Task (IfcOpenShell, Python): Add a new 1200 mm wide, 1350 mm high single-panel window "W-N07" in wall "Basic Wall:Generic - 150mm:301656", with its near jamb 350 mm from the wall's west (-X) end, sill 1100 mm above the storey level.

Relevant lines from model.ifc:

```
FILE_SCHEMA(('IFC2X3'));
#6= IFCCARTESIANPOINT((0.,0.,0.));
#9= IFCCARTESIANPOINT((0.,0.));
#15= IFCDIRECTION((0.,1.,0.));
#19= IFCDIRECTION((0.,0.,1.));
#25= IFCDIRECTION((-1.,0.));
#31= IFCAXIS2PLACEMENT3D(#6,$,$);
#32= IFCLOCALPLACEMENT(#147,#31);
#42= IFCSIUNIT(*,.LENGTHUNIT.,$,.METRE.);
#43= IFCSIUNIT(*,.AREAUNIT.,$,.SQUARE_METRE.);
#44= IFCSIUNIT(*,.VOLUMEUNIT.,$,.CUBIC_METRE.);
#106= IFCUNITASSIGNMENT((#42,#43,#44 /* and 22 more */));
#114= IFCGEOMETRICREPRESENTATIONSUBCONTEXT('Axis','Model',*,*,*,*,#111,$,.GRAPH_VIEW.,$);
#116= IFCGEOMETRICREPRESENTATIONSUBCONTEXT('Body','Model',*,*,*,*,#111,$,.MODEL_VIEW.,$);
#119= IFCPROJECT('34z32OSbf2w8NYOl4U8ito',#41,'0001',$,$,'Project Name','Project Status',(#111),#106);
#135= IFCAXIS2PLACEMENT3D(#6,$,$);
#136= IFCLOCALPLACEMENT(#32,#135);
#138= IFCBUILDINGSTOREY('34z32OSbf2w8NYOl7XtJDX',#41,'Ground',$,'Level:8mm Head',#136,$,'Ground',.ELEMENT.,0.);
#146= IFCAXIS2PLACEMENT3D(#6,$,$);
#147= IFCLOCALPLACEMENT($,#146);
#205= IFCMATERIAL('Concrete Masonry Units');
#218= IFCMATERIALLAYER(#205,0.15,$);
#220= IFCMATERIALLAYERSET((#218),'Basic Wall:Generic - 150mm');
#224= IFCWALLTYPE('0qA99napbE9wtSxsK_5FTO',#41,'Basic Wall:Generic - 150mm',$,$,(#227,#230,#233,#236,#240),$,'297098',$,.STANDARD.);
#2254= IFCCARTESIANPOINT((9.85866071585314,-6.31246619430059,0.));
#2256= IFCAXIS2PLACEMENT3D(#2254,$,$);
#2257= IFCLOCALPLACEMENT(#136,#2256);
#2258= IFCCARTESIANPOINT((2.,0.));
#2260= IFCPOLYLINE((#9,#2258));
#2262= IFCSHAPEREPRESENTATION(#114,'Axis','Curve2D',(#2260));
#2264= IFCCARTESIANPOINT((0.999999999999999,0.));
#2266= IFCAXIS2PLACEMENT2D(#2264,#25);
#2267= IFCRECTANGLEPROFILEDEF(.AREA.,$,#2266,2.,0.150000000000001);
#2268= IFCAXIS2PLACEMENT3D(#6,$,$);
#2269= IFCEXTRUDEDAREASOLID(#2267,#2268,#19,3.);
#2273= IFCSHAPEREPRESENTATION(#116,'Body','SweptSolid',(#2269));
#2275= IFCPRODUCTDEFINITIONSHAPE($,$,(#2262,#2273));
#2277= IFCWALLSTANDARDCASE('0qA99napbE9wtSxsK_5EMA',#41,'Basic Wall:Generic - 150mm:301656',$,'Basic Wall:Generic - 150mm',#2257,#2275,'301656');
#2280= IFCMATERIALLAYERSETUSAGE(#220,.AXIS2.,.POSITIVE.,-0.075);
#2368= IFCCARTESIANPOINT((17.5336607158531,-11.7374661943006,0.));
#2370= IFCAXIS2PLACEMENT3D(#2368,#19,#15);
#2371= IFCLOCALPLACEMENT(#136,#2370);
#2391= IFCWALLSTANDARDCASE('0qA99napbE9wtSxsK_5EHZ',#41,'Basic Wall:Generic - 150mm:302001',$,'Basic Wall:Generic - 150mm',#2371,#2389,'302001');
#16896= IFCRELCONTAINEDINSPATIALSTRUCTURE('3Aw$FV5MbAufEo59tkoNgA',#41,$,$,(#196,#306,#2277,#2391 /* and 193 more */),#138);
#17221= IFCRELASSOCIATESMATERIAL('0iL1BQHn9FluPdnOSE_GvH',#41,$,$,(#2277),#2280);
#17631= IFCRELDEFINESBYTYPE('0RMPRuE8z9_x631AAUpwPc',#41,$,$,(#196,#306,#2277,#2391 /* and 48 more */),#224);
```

```python
import numpy as np
import ifcopenshell
import ifcopenshell.api.feature
import ifcopenshell.api.geometry
import ifcopenshell.api.root
import ifcopenshell.api.spatial
import ifcopenshell.api.type
import ifcopenshell.geom
import ifcopenshell.util.element
import ifcopenshell.util.placement
import ifcopenshell.util.representation
import ifcopenshell.util.shape
import ifcopenshell.util.unit

model = ifcopenshell.open("model.ifc")
unit_scale = ifcopenshell.util.unit.calculate_unit_scale(model)
settings = ifcopenshell.geom.settings()


def volume(element):
    """Net volume in cubic metres, openings subtracted."""
    shape = ifcopenshell.geom.create_shape(settings, element)
    return ifcopenshell.util.shape.get_volume(shape.geometry)


wall = model.by_guid("0qA99napbE9wtSxsK_5EMA")
storey = ifcopenshell.util.element.get_container(wall, ifc_class="IfcBuildingStorey")
context = ifcopenshell.util.representation.get_context(model, "Model", "Body", "MODEL_VIEW")
before = volume(wall)

width, height, from_end, sill = 1.2, 1.35, 0.35, 1.1  # metres

# The wall runs along its own X axis, and the end named is its -X end.
wall_shape = ifcopenshell.geom.create_shape(settings, wall)
x, y, z = ifcopenshell.util.shape.get_vertices(wall_shape.geometry).T
start = x.min() + from_end
face, thickness = float(y.min()), float(y.max() - y.min())
wall_matrix = ifcopenshell.util.placement.get_local_placement(wall.ObjectPlacement)
level = ifcopenshell.util.placement.get_local_placement(storey.ObjectPlacement)[2, 3]


def in_wall(x, y):
    """Placement at x, y metres in the wall's axes, at sill height."""
    matrix = wall_matrix.copy()
    matrix[:, 3] = wall_matrix @ np.array([x / unit_scale, y / unit_scale, 0.0, 1.0])
    matrix[2, 3] = level + sill / unit_scale
    return matrix


# Opening: a box that overshoots both wall faces by 50 mm.
opening = ifcopenshell.api.root.create_entity(model, ifc_class="IfcOpeningElement")
box = ifcopenshell.api.geometry.add_wall_representation(
    model, context=context, length=width, height=height, thickness=thickness + 0.1
)
ifcopenshell.api.geometry.assign_representation(model, product=opening, representation=box)
ifcopenshell.api.geometry.edit_object_placement(model, product=opening, matrix=in_wall(start, face - 0.05), is_si=False)
ifcopenshell.api.feature.add_feature(model, feature=opening, element=wall)

window = ifcopenshell.api.root.create_entity(model, ifc_class="IfcWindow", name="W-N07")
window.OverallWidth, window.OverallHeight = width / unit_scale, height / unit_scale
body = ifcopenshell.api.geometry.add_window_representation(
    model,
    context=context,
    overall_width=window.OverallWidth,
    overall_height=window.OverallHeight,
    partition_type="SINGLE_PANEL",
)
ifcopenshell.api.geometry.assign_representation(model, product=window, representation=body)
ifcopenshell.api.spatial.assign_container(model, products=[window], relating_structure=storey)
fills = ifcopenshell.api.feature.add_filling(model, opening=opening, element=window)
fills.OwnerHistory = window.OwnerHistory  # required in IFC2X3

# IFC2X3 keeps the operation on the window style.
style = ifcopenshell.api.root.create_entity(model, ifc_class="IfcWindowStyle", name="W-N07")
style.OperationType, style.ConstructionType = "SINGLE_PANEL", "NOTDEFINED"
style.ParameterTakesPrecedence = style.Sizeable = False
ifcopenshell.api.type.assign_type(model, related_objects=[window], relating_type=style)

# Centre the window in the wall's thickness.
ifcopenshell.api.geometry.edit_object_placement(model, product=window, matrix=in_wall(start, face), is_si=False)
window_shape = ifcopenshell.geom.create_shape(settings, window)
depth = ifcopenshell.util.shape.get_vertices(window_shape.geometry)[:, 1]
offset = face + thickness / 2 - (depth.min() + depth.max()) / 2
ifcopenshell.api.geometry.edit_object_placement(model, product=window, matrix=in_wall(start, offset), is_si=False)

after = volume(wall)

print(f"wall volume {before:.3f} -> {after:.3f} m3")

model.write("model_updated.ifc")
```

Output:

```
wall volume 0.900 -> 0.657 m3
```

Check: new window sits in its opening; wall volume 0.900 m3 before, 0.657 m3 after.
